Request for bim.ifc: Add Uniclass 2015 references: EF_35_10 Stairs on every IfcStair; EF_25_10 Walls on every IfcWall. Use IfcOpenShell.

First a look at what the model holds.

```python
import ifcopenshell

model = ifcopenshell.open("bim.ifc")
print(model.schema)
print("classifications:", [c.Name for c in model.by_type("IfcClassification")])
for ifc_class in ("IfcDoor", "IfcRoof", "IfcStair", "IfcWall", "IfcWindow"):
    print(ifc_class, len(model.by_type(ifc_class)))
```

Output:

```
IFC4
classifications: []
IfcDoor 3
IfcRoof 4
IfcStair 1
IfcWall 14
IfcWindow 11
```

```python
import ifcopenshell
import ifcopenshell.api.classification

model = ifcopenshell.open("bim.ifc")

system = ifcopenshell.api.classification.add_classification(model, classification="Uniclass 2015")

codes = {
    "IfcStair": ("EF_35_10", "Stairs"),
    "IfcWall": ("EF_25_10", "Walls"),
}
for ifc_class, (code, name) in codes.items():
    products = model.by_type(ifc_class)
    ifcopenshell.api.classification.add_reference(
        model, products=products, classification=system, identification=code, name=name
    )
    print(code, len(products))

model.write("bim_edited.ifc")
```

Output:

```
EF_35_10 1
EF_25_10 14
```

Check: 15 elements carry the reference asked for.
